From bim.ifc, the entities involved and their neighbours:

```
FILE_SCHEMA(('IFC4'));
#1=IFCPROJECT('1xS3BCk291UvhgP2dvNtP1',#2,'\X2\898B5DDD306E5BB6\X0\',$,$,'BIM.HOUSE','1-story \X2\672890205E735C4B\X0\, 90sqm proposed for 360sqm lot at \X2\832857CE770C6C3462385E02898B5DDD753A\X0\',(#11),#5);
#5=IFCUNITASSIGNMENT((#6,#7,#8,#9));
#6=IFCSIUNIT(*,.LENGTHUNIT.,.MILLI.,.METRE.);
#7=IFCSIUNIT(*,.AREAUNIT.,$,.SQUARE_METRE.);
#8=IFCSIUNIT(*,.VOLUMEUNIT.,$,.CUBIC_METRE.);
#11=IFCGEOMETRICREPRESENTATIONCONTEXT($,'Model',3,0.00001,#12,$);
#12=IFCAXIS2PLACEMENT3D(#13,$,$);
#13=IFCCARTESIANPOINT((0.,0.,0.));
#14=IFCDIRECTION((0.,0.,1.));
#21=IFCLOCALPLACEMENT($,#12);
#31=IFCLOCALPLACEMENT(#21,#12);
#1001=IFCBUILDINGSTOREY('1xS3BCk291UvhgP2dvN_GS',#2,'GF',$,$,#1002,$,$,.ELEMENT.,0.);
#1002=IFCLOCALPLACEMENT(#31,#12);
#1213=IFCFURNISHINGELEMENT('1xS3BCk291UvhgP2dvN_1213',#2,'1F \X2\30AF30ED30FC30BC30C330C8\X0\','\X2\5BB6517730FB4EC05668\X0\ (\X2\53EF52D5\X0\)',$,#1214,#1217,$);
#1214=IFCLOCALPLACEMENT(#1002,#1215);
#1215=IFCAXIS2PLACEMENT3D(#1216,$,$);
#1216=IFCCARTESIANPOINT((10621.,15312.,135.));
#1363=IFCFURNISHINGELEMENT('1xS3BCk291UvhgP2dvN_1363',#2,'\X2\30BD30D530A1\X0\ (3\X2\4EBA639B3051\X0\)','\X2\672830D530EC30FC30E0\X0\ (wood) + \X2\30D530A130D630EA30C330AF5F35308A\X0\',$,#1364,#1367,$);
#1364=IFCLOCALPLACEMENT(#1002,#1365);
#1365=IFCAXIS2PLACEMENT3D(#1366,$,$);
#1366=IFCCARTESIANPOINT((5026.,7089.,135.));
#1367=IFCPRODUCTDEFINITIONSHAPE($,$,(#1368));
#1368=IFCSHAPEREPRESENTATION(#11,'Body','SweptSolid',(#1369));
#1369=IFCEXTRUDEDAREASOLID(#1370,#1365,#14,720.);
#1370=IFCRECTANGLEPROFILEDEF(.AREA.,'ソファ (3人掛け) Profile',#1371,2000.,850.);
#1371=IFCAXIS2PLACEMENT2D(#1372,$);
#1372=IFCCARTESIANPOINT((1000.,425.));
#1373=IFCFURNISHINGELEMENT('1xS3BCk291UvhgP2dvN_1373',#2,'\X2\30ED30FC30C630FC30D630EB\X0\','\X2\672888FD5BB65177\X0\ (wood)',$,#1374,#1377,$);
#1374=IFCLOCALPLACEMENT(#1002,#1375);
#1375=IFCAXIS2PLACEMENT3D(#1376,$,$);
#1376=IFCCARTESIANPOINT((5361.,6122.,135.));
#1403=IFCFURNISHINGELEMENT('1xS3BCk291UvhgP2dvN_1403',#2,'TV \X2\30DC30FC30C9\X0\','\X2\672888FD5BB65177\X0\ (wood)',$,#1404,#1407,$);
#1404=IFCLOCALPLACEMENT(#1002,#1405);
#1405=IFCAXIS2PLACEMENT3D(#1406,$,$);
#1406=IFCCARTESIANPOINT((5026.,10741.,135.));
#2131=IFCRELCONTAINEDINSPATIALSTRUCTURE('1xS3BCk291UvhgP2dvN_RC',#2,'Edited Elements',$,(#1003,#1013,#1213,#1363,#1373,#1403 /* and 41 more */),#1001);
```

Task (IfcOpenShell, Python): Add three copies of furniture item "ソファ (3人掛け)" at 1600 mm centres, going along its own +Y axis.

```python
import ifcopenshell
import ifcopenshell.api.geometry
import ifcopenshell.api.root
import ifcopenshell.util.element
import ifcopenshell.util.placement
import ifcopenshell.util.unit

model = ifcopenshell.open("bim.ifc")
unit_scale = ifcopenshell.util.unit.calculate_unit_scale(model)


def reuse_history(source, copy):
    """copy_class also copies each property set's owner history, people and application; keep the originals."""
    for rel in copy.IsDefinedBy:
        if rel.is_a("IfcRelDefinesByProperties") and (history := rel.RelatingPropertyDefinition.OwnerHistory):
            rel.RelatingPropertyDefinition.OwnerHistory = source.OwnerHistory
            ifcopenshell.util.element.remove_deep2(model, history)


source = model.by_id(1363)
base = ifcopenshell.util.placement.get_local_placement(source.ObjectPlacement)
step = base[:3, 1] * 1.6 / unit_scale

for i in range(1, 4):
    copy = ifcopenshell.api.root.copy_class(model, product=source)
    copy.Representation = ifcopenshell.util.element.copy_deep(
        model, source.Representation, exclude=["IfcGeometricRepresentationContext", "IfcRepresentationMap"]
    )
    reuse_history(source, copy)
    matrix = base.copy()
    matrix[:3, 3] += i * step
    print("added at", matrix[:3, 3].round(3) + 0.0)
    ifcopenshell.api.geometry.edit_object_placement(model, product=copy, matrix=matrix, is_si=False)

model.write("bim-out.ifc")
```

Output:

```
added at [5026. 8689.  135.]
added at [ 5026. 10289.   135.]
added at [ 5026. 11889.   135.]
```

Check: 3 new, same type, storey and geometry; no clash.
